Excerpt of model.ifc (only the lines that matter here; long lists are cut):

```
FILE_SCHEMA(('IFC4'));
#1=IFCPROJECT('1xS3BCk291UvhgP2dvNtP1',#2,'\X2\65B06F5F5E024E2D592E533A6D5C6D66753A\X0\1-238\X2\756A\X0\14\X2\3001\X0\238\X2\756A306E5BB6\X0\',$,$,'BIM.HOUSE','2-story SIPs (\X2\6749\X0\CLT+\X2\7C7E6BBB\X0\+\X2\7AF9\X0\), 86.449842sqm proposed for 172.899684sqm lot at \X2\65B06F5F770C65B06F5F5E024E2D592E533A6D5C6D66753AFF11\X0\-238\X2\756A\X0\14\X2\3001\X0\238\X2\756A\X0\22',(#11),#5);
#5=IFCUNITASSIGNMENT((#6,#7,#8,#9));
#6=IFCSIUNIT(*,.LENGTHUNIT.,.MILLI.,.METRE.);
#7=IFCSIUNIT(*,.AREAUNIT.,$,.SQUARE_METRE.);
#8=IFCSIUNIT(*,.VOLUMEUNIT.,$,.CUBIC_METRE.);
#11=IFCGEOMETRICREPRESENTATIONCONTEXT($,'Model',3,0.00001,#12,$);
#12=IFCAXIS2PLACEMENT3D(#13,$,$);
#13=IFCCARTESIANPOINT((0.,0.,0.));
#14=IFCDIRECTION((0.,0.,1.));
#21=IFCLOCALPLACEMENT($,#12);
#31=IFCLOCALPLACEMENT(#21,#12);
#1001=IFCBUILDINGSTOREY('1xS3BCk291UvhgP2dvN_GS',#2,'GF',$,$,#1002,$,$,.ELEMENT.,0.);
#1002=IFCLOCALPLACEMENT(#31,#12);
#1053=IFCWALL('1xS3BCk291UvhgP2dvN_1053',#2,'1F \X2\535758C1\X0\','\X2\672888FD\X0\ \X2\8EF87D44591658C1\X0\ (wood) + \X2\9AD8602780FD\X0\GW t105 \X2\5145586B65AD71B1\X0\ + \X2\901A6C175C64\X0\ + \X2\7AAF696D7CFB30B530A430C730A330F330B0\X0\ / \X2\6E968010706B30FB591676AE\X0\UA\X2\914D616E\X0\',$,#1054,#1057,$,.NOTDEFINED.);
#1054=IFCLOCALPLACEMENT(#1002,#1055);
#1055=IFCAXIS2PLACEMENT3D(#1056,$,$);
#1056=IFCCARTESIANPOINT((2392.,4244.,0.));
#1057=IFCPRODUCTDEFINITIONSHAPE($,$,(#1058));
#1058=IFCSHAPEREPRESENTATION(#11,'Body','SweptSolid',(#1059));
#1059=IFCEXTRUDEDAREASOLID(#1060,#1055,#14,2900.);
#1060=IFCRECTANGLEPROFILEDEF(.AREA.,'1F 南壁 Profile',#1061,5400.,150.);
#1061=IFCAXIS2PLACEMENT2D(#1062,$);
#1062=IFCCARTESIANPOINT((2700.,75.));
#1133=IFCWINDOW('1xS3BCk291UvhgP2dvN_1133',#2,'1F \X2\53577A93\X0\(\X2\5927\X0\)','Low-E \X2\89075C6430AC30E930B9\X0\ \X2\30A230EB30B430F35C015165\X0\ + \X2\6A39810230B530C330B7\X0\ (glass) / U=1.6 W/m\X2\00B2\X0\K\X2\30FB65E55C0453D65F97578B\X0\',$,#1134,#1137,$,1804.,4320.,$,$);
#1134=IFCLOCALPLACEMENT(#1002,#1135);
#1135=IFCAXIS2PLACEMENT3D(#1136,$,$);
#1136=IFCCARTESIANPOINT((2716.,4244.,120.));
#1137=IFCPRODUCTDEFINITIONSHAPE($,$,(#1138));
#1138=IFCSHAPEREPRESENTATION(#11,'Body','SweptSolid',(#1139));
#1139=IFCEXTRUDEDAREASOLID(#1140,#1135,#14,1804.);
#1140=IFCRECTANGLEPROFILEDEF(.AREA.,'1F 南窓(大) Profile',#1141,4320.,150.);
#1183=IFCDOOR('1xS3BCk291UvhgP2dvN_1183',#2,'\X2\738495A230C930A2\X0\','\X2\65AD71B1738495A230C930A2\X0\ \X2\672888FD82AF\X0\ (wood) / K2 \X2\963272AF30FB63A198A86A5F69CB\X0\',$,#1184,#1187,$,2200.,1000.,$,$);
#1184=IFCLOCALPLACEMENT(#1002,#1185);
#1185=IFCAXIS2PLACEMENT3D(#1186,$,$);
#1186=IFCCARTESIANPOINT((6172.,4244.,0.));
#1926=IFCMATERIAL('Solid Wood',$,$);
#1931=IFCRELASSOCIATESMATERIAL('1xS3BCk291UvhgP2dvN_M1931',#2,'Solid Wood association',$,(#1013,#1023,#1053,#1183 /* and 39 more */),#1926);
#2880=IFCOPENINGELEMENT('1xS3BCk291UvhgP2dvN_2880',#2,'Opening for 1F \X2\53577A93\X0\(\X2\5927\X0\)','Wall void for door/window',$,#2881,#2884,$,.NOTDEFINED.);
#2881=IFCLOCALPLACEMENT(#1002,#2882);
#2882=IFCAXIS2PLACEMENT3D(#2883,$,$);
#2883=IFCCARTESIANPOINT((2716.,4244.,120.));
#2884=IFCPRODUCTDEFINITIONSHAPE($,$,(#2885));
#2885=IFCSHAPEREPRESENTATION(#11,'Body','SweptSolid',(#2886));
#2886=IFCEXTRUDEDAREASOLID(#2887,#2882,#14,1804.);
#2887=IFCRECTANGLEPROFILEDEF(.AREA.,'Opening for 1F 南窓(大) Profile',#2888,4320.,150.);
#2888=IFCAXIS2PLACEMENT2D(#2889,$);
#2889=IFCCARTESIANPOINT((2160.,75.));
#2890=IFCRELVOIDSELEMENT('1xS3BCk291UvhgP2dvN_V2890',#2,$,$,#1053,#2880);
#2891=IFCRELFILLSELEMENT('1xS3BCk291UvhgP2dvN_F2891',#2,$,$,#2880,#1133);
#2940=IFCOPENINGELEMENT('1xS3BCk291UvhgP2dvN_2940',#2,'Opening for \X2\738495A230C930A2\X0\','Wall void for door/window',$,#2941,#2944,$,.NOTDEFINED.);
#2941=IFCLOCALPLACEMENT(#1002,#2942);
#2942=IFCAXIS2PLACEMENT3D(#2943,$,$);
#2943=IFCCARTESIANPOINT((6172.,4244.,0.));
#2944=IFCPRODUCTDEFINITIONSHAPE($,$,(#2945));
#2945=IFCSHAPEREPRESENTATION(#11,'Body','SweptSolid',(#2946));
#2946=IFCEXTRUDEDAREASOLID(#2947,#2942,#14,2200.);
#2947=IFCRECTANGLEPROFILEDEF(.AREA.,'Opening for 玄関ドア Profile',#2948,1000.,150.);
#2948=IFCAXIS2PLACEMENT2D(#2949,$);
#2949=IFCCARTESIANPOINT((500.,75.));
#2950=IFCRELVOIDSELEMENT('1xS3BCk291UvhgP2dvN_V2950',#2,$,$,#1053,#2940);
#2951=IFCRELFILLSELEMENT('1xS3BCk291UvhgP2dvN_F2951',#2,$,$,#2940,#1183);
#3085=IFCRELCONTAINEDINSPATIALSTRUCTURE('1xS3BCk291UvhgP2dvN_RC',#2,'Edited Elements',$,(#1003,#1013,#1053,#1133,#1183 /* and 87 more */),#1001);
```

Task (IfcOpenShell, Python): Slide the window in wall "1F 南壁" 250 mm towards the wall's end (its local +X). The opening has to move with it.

```python
import ifcopenshell
import ifcopenshell.api.geometry
import ifcopenshell.util.placement
import ifcopenshell.util.unit

model = ifcopenshell.open("model.ifc")
unit_scale = ifcopenshell.util.unit.calculate_unit_scale(model)

window = model.by_guid("1xS3BCk291UvhgP2dvN_1133")
opening = window.FillsVoids[0].RelatingOpeningElement
wall = opening.VoidsElements[0].RelatingBuildingElement

wall_matrix = ifcopenshell.util.placement.get_local_placement(wall.ObjectPlacement)
shift = wall_matrix[:3, 0] * 0.25 / unit_scale
before = ifcopenshell.util.placement.get_local_placement(window.ObjectPlacement)[:3, 3].copy()

# The window is not placed relative to its opening, so move both.
for product in (opening, window):
    matrix = ifcopenshell.util.placement.get_local_placement(product.ObjectPlacement)
    matrix[:3, 3] += shift
    ifcopenshell.api.geometry.edit_object_placement(model, product=product, matrix=matrix, is_si=False)

after = ifcopenshell.util.placement.get_local_placement(window.ObjectPlacement)[:3, 3]
print("window moved by", (after - before).round(3) + 0.0)

model.write("model_edited.ifc")
```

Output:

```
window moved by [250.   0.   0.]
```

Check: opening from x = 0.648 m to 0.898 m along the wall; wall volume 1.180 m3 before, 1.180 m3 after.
